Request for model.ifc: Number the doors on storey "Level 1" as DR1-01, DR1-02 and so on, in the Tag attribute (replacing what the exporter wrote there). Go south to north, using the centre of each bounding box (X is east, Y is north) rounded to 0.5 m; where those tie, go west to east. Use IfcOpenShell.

First a look at what the model holds.

```python
import ifcopenshell
import ifcopenshell.util.element
import ifcopenshell.util.placement

model = ifcopenshell.open("model.ifc")
print(model.schema)
storey = next(s for s in model.by_type("IfcBuildingStorey") if s.Name == "Level 1")
doors = [e for e in ifcopenshell.util.element.get_decomposition(storey) if e.is_a("IfcDoor")]
for e in sorted(doors, key=lambda e: e.id()):
    origin = ifcopenshell.util.placement.get_local_placement(e.ObjectPlacement)[:3, 3]
    print(e.id(), e.Tag, e.Name, origin.round(2) + 0.0, sep=" | ")
```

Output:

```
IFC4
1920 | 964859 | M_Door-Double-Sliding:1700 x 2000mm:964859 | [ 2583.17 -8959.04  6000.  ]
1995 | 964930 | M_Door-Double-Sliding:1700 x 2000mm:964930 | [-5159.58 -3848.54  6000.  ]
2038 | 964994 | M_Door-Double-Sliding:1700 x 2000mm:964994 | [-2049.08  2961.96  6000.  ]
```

```python
import ifcopenshell
import ifcopenshell.geom
import ifcopenshell.util.element
import ifcopenshell.util.shape

model = ifcopenshell.open("model.ifc")
settings = ifcopenshell.geom.settings()
settings.set("use-world-coords", True)


def centre(element):
    shape = ifcopenshell.geom.create_shape(settings, element)
    return ifcopenshell.util.shape.get_bbox_centroid(shape.geometry)


storey = next(s for s in model.by_type("IfcBuildingStorey") if s.Name == "Level 1")
doors = [e for e in ifcopenshell.util.element.get_decomposition(storey) if e.is_a("IfcDoor")]

# Insertion points can sit at a corner or the storey origin, so sort by the geometry (in metres).
centres = {e: centre(e) for e in doors}
doors.sort(key=lambda e: (round(centres[e][1] / 0.5), centres[e][0]))

for i, e in enumerate(doors, start=1):
    number = f"DR1-{i:02d}"
    e.Tag = number
    print(e.id(), number)

model.write("model_v2.ifc")
```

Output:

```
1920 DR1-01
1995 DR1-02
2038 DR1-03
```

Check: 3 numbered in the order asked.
